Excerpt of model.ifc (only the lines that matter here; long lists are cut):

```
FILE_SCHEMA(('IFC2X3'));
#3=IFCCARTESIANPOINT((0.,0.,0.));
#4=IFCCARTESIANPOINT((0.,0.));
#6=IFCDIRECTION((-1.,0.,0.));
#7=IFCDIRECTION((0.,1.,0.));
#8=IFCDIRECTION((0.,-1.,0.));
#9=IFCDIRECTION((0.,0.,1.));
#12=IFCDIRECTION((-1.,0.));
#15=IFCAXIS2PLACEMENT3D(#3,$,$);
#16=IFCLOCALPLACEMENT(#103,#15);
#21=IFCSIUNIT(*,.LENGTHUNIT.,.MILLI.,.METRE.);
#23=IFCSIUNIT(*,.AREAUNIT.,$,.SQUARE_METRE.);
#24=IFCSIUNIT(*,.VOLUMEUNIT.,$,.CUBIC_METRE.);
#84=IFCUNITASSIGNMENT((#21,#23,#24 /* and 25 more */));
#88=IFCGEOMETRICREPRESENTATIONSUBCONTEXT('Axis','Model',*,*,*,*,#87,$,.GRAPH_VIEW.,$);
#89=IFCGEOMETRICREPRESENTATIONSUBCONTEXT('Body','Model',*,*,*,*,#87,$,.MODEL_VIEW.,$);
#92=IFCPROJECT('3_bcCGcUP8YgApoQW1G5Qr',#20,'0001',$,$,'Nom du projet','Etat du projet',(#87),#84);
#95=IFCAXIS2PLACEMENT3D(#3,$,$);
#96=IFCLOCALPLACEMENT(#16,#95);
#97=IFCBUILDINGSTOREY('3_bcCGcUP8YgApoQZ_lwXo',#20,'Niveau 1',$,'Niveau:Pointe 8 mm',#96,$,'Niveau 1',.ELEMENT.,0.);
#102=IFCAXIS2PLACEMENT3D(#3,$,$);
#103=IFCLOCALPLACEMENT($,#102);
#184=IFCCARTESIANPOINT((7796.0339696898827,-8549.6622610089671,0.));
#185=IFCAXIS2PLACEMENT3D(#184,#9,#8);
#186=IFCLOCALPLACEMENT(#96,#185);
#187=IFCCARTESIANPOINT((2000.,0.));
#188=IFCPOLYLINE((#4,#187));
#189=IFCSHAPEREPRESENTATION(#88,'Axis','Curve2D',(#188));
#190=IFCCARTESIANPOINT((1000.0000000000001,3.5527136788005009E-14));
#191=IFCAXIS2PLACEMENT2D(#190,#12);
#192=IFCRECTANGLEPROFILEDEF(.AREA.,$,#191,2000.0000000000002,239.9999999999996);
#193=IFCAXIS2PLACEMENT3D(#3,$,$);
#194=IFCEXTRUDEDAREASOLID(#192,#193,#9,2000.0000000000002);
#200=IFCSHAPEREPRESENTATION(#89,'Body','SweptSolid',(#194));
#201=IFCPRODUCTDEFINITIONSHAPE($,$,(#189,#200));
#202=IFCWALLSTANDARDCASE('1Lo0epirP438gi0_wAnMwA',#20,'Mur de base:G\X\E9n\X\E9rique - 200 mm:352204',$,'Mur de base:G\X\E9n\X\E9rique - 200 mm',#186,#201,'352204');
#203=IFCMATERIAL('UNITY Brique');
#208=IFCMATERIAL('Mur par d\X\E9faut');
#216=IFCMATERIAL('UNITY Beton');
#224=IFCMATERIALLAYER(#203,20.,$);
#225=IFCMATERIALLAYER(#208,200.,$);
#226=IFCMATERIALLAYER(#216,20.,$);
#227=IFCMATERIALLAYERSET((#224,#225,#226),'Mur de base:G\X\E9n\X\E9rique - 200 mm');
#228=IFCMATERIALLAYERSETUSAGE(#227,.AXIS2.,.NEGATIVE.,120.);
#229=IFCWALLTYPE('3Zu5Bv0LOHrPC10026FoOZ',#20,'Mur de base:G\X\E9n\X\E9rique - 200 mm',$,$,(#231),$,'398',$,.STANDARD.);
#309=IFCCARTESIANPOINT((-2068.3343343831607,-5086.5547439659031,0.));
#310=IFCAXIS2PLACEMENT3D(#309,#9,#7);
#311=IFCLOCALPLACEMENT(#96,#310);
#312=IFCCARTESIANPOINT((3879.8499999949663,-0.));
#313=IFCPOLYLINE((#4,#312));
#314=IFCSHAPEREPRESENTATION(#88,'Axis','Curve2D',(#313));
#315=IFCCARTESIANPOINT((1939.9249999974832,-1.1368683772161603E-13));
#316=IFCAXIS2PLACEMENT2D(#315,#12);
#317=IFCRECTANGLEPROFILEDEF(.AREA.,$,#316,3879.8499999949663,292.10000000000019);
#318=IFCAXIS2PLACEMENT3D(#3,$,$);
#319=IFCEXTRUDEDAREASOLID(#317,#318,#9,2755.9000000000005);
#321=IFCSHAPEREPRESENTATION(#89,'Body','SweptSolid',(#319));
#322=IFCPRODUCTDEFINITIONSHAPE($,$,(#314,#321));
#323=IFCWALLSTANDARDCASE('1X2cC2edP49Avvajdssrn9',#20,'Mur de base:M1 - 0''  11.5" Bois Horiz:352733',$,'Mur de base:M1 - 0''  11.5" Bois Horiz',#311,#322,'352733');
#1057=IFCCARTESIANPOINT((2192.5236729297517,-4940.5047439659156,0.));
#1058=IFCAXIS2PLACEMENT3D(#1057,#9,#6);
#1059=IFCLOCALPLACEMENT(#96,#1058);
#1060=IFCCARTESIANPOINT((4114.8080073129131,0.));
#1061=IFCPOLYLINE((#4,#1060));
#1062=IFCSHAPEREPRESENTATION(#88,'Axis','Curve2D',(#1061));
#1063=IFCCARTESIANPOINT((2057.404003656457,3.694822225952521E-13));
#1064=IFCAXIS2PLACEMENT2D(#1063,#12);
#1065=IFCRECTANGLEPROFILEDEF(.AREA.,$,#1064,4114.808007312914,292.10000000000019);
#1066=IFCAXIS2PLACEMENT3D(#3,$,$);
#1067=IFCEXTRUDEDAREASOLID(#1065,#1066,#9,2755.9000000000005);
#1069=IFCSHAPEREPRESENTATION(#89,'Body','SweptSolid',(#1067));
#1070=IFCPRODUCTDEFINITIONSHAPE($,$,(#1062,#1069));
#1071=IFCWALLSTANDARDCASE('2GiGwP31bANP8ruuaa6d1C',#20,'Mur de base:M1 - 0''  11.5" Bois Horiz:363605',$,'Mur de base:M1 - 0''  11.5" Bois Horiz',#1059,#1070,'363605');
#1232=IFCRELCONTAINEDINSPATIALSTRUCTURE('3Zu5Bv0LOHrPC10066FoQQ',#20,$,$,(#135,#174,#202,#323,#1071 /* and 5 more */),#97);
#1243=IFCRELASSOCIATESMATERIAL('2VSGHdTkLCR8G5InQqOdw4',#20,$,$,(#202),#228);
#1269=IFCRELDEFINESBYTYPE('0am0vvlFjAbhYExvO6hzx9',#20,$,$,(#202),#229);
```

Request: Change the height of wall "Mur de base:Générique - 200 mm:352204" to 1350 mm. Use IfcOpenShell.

```python
import ifcopenshell
import ifcopenshell.geom
import ifcopenshell.util.representation
import ifcopenshell.util.shape

model = ifcopenshell.open("model.ifc")
settings = ifcopenshell.geom.settings()


def volume(element):
    """Net volume in cubic metres, openings subtracted."""
    shape = ifcopenshell.geom.create_shape(settings, element)
    return ifcopenshell.util.shape.get_volume(shape.geometry)


wall = model.by_guid("1Lo0epirP438gi0_wAnMwA")
before = volume(wall)

body = ifcopenshell.util.representation.get_representation(wall, "Model", "Body")
solid = body.Items[0]
old_height = solid.Depth
solid.Depth = 1350.0
after = volume(wall)

print(f"height {old_height:g} -> {solid.Depth:g}, volume {before:.3f} -> {after:.3f} m3")

model.write("model_edited.ifc")
```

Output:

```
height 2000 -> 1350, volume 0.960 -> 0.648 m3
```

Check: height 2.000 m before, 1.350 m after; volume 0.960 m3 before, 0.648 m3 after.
